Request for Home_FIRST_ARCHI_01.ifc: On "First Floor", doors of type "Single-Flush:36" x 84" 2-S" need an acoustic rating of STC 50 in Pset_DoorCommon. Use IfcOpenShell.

First a look at what the model holds.

```python
import ifcopenshell
import ifcopenshell.util.element

model = ifcopenshell.open("Home_FIRST_ARCHI_01.ifc")
print(model.schema)
storey = next(s for s in model.by_type("IfcBuildingStorey") if s.Name == "First Floor")
doors = [e for e in ifcopenshell.util.element.get_decomposition(storey) if e.is_a("IfcDoor")]
seen = {}
for e in doors:
    element_type = ifcopenshell.util.element.get_type(e)
    key = (element_type.Name if element_type != e and element_type else None, ifcopenshell.util.element.get_pset(e, "Pset_DoorCommon", "AcousticRating"))
    seen[key] = seen.get(key, 0) + 1
for (name, value), count in sorted(seen.items(), key=str):
    print(count, "x", name, "|", value)
```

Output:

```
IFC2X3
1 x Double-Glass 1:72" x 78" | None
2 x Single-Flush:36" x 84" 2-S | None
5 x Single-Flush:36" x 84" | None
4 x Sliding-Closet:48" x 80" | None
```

```python
import ifcopenshell
import ifcopenshell.api.pset
import ifcopenshell.util.element

model = ifcopenshell.open("Home_FIRST_ARCHI_01.ifc")

storey = next(s for s in model.by_type("IfcBuildingStorey") if s.Name == "First Floor")
doors = [e for e in ifcopenshell.util.element.get_decomposition(storey) if e.is_a("IfcDoor")]

count = 0
for e in doors:
    element_type = ifcopenshell.util.element.get_type(e)
    if element_type in (None, e) or element_type.Name != 'Single-Flush:36" x 84" 2-S':
        continue
    # add_pset returns the element's existing set when there is one.
    pset = ifcopenshell.api.pset.add_pset(model, product=e, name="Pset_DoorCommon")
    ifcopenshell.api.pset.edit_pset(model, pset=pset, properties={"AcousticRating": "STC 50"})
    count += 1

print(count, "doors updated")

model.write("Home_FIRST_ARCHI_01_updated.ifc")
```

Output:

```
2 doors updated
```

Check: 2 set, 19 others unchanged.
